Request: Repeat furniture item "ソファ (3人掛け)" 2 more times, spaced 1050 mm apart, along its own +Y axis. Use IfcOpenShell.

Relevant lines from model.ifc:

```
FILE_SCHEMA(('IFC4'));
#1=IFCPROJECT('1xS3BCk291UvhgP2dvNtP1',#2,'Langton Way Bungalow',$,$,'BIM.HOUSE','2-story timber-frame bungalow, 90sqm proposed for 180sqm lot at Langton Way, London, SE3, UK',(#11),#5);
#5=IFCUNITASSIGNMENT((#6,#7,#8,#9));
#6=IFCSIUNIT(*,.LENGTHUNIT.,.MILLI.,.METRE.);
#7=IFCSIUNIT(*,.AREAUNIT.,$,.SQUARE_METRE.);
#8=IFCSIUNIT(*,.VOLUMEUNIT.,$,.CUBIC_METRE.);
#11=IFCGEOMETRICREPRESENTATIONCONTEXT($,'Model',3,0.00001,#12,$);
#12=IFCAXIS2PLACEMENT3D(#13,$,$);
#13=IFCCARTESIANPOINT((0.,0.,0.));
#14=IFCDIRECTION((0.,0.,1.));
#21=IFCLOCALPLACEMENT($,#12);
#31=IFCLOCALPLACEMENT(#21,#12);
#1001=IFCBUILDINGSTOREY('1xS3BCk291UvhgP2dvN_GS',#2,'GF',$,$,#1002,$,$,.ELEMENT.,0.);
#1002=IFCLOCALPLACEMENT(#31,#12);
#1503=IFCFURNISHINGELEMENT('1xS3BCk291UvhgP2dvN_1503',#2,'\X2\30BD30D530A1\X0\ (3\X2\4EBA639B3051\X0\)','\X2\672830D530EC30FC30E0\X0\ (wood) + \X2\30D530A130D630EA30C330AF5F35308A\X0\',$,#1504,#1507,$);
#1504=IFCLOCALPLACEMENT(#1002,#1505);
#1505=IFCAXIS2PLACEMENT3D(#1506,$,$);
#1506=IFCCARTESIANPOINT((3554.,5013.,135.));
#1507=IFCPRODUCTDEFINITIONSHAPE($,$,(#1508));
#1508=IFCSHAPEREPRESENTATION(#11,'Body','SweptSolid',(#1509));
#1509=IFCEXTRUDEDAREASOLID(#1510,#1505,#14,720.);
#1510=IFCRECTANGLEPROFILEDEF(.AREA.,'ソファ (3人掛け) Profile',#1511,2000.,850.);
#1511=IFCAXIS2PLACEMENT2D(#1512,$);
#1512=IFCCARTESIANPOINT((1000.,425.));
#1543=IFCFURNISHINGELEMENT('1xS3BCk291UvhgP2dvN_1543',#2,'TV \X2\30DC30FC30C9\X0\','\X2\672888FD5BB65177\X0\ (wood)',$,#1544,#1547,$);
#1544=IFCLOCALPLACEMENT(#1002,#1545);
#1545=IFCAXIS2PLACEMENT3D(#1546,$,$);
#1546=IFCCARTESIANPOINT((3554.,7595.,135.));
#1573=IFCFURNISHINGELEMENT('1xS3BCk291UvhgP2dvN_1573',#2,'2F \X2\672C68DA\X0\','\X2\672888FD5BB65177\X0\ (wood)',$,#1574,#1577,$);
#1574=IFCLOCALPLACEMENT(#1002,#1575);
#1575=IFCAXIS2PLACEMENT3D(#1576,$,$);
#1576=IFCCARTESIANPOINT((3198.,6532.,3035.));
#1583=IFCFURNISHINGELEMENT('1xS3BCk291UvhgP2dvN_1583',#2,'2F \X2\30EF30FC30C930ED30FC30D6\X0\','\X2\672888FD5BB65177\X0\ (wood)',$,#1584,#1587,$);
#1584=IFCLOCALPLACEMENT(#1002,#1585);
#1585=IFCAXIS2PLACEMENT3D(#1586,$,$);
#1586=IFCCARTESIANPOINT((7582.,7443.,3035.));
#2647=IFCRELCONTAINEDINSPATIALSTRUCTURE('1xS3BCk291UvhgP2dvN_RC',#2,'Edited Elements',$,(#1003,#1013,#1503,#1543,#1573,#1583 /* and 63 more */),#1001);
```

```python
import ifcopenshell
import ifcopenshell.api.geometry
import ifcopenshell.api.root
import ifcopenshell.util.element
import ifcopenshell.util.placement

model = ifcopenshell.open("model.ifc")


def reuse_history(source, copy):
    """copy_class also copies each property set's owner history, people and application; keep the originals."""
    for rel in copy.IsDefinedBy:
        if rel.is_a("IfcRelDefinesByProperties") and (history := rel.RelatingPropertyDefinition.OwnerHistory):
            rel.RelatingPropertyDefinition.OwnerHistory = source.OwnerHistory
            ifcopenshell.util.element.remove_deep2(model, history)


source = model.by_guid("1xS3BCk291UvhgP2dvN_1503")
base = ifcopenshell.util.placement.get_local_placement(source.ObjectPlacement)
step = base[:3, 1] * 1050.0

for i in range(1, 3):
    copy = ifcopenshell.api.root.copy_class(model, product=source)
    copy.Representation = ifcopenshell.util.element.copy_deep(
        model, source.Representation, exclude=["IfcGeometricRepresentationContext", "IfcRepresentationMap"]
    )
    reuse_history(source, copy)
    matrix = base.copy()
    matrix[:3, 3] += i * step
    print("added at", matrix[:3, 3].round(3) + 0.0)
    ifcopenshell.api.geometry.edit_object_placement(model, product=copy, matrix=matrix, is_si=False)

model.write("model-out.ifc")
```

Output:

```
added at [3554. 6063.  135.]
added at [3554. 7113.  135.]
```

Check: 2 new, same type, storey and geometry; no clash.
